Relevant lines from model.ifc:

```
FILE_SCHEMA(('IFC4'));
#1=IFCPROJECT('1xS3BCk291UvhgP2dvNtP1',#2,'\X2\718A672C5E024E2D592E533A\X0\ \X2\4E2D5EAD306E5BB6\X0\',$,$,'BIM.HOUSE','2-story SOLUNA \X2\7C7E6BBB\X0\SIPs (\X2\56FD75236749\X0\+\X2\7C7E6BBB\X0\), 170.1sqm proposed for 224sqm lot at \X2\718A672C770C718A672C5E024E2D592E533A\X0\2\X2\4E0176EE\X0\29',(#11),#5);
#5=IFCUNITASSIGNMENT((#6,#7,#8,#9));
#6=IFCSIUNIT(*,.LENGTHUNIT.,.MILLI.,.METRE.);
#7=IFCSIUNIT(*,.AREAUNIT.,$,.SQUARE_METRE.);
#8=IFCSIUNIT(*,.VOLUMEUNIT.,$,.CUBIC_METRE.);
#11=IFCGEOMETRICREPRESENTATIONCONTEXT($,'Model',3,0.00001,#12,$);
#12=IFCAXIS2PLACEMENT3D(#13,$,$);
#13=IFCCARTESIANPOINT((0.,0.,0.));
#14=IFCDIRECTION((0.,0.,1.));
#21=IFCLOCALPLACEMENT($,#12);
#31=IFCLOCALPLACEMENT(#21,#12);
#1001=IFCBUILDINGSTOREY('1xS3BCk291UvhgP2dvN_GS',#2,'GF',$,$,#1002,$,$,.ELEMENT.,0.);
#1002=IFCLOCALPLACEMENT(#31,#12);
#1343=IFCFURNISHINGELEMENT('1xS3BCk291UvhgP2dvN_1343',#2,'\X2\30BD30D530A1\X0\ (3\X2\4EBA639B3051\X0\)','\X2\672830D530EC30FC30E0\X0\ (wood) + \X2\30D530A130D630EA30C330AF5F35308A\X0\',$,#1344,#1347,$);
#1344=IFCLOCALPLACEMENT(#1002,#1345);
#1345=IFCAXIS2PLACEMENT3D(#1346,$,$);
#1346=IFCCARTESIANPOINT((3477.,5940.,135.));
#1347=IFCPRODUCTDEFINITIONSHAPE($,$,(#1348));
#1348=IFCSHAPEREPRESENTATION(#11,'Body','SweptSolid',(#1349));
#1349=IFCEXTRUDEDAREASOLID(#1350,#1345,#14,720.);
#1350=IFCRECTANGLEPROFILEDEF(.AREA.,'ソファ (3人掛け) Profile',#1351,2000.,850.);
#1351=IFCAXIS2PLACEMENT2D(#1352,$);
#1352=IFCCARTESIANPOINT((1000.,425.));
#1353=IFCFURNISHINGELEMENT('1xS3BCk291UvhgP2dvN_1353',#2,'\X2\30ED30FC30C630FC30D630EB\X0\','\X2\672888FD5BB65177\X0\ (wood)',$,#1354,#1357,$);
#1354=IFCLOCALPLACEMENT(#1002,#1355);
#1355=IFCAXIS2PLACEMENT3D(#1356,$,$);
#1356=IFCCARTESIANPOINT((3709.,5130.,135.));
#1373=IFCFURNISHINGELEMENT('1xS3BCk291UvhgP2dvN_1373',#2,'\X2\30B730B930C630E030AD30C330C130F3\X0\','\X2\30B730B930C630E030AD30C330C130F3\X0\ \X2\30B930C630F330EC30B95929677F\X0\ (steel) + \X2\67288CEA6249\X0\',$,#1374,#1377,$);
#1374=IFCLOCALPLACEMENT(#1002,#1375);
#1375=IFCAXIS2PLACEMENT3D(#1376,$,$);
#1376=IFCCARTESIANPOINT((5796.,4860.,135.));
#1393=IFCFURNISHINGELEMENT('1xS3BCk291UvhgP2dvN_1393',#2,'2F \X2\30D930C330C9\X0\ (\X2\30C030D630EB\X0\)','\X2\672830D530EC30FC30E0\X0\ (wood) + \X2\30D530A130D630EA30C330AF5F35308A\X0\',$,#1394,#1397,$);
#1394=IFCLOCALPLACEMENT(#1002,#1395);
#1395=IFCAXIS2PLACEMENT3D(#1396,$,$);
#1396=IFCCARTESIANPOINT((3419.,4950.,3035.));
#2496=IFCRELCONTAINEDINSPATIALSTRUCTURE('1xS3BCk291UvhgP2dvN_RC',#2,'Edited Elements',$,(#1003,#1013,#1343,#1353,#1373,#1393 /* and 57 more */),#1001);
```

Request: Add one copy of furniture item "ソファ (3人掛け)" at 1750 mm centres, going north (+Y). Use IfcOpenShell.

```python
import numpy as np
import ifcopenshell
import ifcopenshell.api.geometry
import ifcopenshell.api.root
import ifcopenshell.util.element
import ifcopenshell.util.placement

model = ifcopenshell.open("model.ifc")


def reuse_history(source, copy):
    """copy_class also copies each property set's owner history, people and application; keep the originals."""
    for rel in copy.IsDefinedBy:
        if rel.is_a("IfcRelDefinesByProperties") and (history := rel.RelatingPropertyDefinition.OwnerHistory):
            rel.RelatingPropertyDefinition.OwnerHistory = source.OwnerHistory
            ifcopenshell.util.element.remove_deep2(model, history)


source = model.by_guid("1xS3BCk291UvhgP2dvN_1343")
base = ifcopenshell.util.placement.get_local_placement(source.ObjectPlacement)
step = np.array([0.0, 1.0, 0.0]) * 1750.0

for i in range(1, 2):
    copy = ifcopenshell.api.root.copy_class(model, product=source)
    copy.Representation = ifcopenshell.util.element.copy_deep(
        model, source.Representation, exclude=["IfcGeometricRepresentationContext", "IfcRepresentationMap"]
    )
    reuse_history(source, copy)
    matrix = base.copy()
    matrix[:3, 3] += i * step
    print("added at", matrix[:3, 3].round(3) + 0.0)
    ifcopenshell.api.geometry.edit_object_placement(model, product=copy, matrix=matrix, is_si=False)

model.write("model-out.ifc")
```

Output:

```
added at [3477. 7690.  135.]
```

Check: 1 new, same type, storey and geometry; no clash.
